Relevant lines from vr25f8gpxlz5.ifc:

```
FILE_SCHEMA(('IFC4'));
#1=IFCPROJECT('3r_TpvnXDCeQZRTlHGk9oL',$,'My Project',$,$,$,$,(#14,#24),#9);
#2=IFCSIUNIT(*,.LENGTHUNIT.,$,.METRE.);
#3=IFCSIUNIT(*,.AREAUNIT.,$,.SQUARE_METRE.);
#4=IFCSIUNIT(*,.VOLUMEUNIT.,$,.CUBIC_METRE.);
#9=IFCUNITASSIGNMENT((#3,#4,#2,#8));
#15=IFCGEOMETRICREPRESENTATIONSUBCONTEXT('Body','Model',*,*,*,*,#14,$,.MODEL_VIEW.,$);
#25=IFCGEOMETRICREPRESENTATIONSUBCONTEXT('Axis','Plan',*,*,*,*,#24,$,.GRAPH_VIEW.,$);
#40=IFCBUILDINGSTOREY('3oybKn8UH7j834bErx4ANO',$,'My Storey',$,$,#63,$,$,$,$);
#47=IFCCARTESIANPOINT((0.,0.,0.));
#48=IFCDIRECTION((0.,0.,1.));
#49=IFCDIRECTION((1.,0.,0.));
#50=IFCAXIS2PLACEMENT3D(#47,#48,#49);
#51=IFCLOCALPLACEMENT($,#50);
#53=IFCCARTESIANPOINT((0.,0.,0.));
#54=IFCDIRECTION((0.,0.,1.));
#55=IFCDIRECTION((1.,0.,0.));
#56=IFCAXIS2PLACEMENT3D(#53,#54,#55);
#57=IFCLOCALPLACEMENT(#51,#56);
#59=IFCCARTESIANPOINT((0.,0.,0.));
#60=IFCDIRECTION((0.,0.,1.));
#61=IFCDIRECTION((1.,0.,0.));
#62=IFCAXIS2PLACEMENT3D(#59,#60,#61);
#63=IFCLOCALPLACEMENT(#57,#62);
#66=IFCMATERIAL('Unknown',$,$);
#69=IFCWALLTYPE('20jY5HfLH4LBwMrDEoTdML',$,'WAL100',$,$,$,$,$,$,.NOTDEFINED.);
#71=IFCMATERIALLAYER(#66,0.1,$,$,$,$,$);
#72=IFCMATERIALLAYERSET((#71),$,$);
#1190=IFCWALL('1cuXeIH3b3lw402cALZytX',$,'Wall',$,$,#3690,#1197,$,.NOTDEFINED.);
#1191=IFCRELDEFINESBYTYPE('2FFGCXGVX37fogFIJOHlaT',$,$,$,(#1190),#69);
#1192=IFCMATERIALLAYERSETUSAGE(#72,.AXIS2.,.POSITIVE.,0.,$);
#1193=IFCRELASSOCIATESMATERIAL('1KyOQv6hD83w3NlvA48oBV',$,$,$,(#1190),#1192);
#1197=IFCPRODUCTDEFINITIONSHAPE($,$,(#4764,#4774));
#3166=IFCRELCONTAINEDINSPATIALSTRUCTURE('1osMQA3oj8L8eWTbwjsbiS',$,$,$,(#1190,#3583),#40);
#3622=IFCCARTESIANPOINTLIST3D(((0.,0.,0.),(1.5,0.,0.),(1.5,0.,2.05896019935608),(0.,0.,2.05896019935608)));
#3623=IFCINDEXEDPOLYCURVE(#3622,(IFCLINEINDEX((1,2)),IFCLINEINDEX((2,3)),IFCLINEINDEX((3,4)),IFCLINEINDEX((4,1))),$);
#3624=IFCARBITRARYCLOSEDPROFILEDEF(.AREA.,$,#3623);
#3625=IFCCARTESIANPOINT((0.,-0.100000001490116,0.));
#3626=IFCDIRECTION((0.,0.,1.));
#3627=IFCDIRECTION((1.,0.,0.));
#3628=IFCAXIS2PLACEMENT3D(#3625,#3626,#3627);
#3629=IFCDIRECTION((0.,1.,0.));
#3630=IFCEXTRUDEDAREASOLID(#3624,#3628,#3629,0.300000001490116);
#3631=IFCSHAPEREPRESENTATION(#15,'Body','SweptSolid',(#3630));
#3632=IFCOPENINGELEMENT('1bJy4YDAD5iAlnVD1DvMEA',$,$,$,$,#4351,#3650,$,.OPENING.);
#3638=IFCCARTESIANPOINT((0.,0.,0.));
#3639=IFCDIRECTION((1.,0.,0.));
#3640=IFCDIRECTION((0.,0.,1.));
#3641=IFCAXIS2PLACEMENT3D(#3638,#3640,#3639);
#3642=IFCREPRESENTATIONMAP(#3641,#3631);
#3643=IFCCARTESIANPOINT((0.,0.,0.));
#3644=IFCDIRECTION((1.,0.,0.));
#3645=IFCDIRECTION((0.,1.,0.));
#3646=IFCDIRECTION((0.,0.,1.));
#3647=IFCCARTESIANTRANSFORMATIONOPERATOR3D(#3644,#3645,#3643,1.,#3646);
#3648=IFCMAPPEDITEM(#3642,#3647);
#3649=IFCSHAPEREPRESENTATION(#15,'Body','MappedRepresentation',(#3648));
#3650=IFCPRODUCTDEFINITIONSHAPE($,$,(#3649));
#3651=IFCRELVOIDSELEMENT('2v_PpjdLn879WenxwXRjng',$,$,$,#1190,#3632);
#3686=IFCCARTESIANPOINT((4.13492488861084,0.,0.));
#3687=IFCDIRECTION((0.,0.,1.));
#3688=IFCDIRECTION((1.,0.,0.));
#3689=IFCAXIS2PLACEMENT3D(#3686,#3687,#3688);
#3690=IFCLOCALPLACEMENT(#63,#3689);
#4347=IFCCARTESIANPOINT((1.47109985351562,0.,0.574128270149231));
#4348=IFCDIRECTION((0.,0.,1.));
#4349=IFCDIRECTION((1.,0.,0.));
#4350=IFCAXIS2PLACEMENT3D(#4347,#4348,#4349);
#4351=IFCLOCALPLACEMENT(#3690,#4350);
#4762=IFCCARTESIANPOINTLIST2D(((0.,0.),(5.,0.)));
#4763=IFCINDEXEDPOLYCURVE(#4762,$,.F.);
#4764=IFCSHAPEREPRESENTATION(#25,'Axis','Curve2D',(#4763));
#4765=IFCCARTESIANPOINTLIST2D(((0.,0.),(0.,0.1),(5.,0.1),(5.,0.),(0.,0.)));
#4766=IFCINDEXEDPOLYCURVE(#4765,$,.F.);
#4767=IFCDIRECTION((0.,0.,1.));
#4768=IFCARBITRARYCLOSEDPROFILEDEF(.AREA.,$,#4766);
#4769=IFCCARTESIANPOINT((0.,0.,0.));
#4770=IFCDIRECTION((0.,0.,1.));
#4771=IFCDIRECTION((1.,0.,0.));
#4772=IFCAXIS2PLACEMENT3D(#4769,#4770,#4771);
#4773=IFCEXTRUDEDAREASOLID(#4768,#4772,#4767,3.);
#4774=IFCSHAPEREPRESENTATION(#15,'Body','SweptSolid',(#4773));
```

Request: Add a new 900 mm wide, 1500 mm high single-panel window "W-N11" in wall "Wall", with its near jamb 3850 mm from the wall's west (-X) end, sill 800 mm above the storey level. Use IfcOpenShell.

```python
import numpy as np
import ifcopenshell
import ifcopenshell.api.feature
import ifcopenshell.api.geometry
import ifcopenshell.api.root
import ifcopenshell.api.spatial
import ifcopenshell.geom
import ifcopenshell.util.element
import ifcopenshell.util.placement
import ifcopenshell.util.representation
import ifcopenshell.util.shape
import ifcopenshell.util.unit

model = ifcopenshell.open("vr25f8gpxlz5.ifc")
unit_scale = ifcopenshell.util.unit.calculate_unit_scale(model)
settings = ifcopenshell.geom.settings()


def volume(element):
    """Net volume in cubic metres, openings subtracted."""
    shape = ifcopenshell.geom.create_shape(settings, element)
    return ifcopenshell.util.shape.get_volume(shape.geometry)


wall = model.by_guid("1cuXeIH3b3lw402cALZytX")
storey = ifcopenshell.util.element.get_container(wall, ifc_class="IfcBuildingStorey")
context = ifcopenshell.util.representation.get_context(model, "Model", "Body", "MODEL_VIEW")
before = volume(wall)

width, height, from_end, sill = 0.9, 1.5, 3.85, 0.8  # metres

# The wall runs along its own X axis, and the end named is its -X end.
wall_shape = ifcopenshell.geom.create_shape(settings, wall)
x, y, z = ifcopenshell.util.shape.get_vertices(wall_shape.geometry).T
start = x.min() + from_end
face, thickness = float(y.min()), float(y.max() - y.min())
wall_matrix = ifcopenshell.util.placement.get_local_placement(wall.ObjectPlacement)
level = ifcopenshell.util.placement.get_local_placement(storey.ObjectPlacement)[2, 3]


def in_wall(x, y):
    """Placement at x, y metres in the wall's axes, at sill height."""
    matrix = wall_matrix.copy()
    matrix[:, 3] = wall_matrix @ np.array([x / unit_scale, y / unit_scale, 0.0, 1.0])
    matrix[2, 3] = level + sill / unit_scale
    return matrix


# Opening: a box that overshoots both wall faces by 50 mm.
opening = ifcopenshell.api.root.create_entity(model, ifc_class="IfcOpeningElement", predefined_type="OPENING")
box = ifcopenshell.api.geometry.add_wall_representation(
    model, context=context, length=width, height=height, thickness=thickness + 0.1
)
ifcopenshell.api.geometry.assign_representation(model, product=opening, representation=box)
ifcopenshell.api.geometry.edit_object_placement(model, product=opening, matrix=in_wall(start, face - 0.05), is_si=False)
ifcopenshell.api.feature.add_feature(model, feature=opening, element=wall)

window = ifcopenshell.api.root.create_entity(model, ifc_class="IfcWindow", name="W-N11", predefined_type="WINDOW")
window.OverallWidth, window.OverallHeight = width / unit_scale, height / unit_scale
window.PartitioningType = "SINGLE_PANEL"
body = ifcopenshell.api.geometry.add_window_representation(
    model,
    context=context,
    overall_width=window.OverallWidth,
    overall_height=window.OverallHeight,
    partition_type="SINGLE_PANEL",
)
ifcopenshell.api.geometry.assign_representation(model, product=window, representation=body)
ifcopenshell.api.spatial.assign_container(model, products=[window], relating_structure=storey)
ifcopenshell.api.feature.add_filling(model, opening=opening, element=window)

# Centre the window in the wall's thickness.
ifcopenshell.api.geometry.edit_object_placement(model, product=window, matrix=in_wall(start, face), is_si=False)
window_shape = ifcopenshell.geom.create_shape(settings, window)
depth = ifcopenshell.util.shape.get_vertices(window_shape.geometry)[:, 1]
offset = face + thickness / 2 - (depth.min() + depth.max()) / 2
ifcopenshell.api.geometry.edit_object_placement(model, product=window, matrix=in_wall(start, offset), is_si=False)

after = volume(wall)

print(f"wall volume {before:.3f} -> {after:.3f} m3")

model.write("vr25f8gpxlz5_v2.ifc")
```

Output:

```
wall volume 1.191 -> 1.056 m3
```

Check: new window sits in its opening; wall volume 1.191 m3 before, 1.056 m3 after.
